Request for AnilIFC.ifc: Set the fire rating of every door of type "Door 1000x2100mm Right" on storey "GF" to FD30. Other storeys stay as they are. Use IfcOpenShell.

First a look at what the model holds.

```python
import ifcopenshell
import ifcopenshell.util.element

model = ifcopenshell.open("AnilIFC.ifc")
print(model.schema)
storey = next(s for s in model.by_type("IfcBuildingStorey") if s.Name == "GF")
doors = [e for e in ifcopenshell.util.element.get_decomposition(storey) if e.is_a("IfcDoor")]
seen = {}
for e in doors:
    element_type = ifcopenshell.util.element.get_type(e)
    key = (element_type.Name if element_type != e and element_type else None, ifcopenshell.util.element.get_pset(e, "Pset_DoorCommon", "FireRating"))
    seen[key] = seen.get(key, 0) + 1
for (name, value), count in sorted(seen.items(), key=str):
    print(count, "x", name, "|", value)
```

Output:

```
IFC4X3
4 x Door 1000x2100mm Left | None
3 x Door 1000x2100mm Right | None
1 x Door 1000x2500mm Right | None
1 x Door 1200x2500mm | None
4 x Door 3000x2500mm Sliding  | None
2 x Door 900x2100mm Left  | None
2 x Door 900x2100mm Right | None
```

```python
import ifcopenshell
import ifcopenshell.api.pset
import ifcopenshell.util.element

model = ifcopenshell.open("AnilIFC.ifc")

storey = next(s for s in model.by_type("IfcBuildingStorey") if s.Name == "GF")
doors = [e for e in ifcopenshell.util.element.get_decomposition(storey) if e.is_a("IfcDoor")]

count = 0
for e in doors:
    element_type = ifcopenshell.util.element.get_type(e)
    if element_type in (None, e) or element_type.Name != "Door 1000x2100mm Right":
        continue
    # add_pset returns the element's existing set when there is one.
    pset = ifcopenshell.api.pset.add_pset(model, product=e, name="Pset_DoorCommon")
    ifcopenshell.api.pset.edit_pset(model, pset=pset, properties={"FireRating": "FD30"})
    count += 1

print(count, "doors updated")

model.write("AnilIFC_edited.ifc")
```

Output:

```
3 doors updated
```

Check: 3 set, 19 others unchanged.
